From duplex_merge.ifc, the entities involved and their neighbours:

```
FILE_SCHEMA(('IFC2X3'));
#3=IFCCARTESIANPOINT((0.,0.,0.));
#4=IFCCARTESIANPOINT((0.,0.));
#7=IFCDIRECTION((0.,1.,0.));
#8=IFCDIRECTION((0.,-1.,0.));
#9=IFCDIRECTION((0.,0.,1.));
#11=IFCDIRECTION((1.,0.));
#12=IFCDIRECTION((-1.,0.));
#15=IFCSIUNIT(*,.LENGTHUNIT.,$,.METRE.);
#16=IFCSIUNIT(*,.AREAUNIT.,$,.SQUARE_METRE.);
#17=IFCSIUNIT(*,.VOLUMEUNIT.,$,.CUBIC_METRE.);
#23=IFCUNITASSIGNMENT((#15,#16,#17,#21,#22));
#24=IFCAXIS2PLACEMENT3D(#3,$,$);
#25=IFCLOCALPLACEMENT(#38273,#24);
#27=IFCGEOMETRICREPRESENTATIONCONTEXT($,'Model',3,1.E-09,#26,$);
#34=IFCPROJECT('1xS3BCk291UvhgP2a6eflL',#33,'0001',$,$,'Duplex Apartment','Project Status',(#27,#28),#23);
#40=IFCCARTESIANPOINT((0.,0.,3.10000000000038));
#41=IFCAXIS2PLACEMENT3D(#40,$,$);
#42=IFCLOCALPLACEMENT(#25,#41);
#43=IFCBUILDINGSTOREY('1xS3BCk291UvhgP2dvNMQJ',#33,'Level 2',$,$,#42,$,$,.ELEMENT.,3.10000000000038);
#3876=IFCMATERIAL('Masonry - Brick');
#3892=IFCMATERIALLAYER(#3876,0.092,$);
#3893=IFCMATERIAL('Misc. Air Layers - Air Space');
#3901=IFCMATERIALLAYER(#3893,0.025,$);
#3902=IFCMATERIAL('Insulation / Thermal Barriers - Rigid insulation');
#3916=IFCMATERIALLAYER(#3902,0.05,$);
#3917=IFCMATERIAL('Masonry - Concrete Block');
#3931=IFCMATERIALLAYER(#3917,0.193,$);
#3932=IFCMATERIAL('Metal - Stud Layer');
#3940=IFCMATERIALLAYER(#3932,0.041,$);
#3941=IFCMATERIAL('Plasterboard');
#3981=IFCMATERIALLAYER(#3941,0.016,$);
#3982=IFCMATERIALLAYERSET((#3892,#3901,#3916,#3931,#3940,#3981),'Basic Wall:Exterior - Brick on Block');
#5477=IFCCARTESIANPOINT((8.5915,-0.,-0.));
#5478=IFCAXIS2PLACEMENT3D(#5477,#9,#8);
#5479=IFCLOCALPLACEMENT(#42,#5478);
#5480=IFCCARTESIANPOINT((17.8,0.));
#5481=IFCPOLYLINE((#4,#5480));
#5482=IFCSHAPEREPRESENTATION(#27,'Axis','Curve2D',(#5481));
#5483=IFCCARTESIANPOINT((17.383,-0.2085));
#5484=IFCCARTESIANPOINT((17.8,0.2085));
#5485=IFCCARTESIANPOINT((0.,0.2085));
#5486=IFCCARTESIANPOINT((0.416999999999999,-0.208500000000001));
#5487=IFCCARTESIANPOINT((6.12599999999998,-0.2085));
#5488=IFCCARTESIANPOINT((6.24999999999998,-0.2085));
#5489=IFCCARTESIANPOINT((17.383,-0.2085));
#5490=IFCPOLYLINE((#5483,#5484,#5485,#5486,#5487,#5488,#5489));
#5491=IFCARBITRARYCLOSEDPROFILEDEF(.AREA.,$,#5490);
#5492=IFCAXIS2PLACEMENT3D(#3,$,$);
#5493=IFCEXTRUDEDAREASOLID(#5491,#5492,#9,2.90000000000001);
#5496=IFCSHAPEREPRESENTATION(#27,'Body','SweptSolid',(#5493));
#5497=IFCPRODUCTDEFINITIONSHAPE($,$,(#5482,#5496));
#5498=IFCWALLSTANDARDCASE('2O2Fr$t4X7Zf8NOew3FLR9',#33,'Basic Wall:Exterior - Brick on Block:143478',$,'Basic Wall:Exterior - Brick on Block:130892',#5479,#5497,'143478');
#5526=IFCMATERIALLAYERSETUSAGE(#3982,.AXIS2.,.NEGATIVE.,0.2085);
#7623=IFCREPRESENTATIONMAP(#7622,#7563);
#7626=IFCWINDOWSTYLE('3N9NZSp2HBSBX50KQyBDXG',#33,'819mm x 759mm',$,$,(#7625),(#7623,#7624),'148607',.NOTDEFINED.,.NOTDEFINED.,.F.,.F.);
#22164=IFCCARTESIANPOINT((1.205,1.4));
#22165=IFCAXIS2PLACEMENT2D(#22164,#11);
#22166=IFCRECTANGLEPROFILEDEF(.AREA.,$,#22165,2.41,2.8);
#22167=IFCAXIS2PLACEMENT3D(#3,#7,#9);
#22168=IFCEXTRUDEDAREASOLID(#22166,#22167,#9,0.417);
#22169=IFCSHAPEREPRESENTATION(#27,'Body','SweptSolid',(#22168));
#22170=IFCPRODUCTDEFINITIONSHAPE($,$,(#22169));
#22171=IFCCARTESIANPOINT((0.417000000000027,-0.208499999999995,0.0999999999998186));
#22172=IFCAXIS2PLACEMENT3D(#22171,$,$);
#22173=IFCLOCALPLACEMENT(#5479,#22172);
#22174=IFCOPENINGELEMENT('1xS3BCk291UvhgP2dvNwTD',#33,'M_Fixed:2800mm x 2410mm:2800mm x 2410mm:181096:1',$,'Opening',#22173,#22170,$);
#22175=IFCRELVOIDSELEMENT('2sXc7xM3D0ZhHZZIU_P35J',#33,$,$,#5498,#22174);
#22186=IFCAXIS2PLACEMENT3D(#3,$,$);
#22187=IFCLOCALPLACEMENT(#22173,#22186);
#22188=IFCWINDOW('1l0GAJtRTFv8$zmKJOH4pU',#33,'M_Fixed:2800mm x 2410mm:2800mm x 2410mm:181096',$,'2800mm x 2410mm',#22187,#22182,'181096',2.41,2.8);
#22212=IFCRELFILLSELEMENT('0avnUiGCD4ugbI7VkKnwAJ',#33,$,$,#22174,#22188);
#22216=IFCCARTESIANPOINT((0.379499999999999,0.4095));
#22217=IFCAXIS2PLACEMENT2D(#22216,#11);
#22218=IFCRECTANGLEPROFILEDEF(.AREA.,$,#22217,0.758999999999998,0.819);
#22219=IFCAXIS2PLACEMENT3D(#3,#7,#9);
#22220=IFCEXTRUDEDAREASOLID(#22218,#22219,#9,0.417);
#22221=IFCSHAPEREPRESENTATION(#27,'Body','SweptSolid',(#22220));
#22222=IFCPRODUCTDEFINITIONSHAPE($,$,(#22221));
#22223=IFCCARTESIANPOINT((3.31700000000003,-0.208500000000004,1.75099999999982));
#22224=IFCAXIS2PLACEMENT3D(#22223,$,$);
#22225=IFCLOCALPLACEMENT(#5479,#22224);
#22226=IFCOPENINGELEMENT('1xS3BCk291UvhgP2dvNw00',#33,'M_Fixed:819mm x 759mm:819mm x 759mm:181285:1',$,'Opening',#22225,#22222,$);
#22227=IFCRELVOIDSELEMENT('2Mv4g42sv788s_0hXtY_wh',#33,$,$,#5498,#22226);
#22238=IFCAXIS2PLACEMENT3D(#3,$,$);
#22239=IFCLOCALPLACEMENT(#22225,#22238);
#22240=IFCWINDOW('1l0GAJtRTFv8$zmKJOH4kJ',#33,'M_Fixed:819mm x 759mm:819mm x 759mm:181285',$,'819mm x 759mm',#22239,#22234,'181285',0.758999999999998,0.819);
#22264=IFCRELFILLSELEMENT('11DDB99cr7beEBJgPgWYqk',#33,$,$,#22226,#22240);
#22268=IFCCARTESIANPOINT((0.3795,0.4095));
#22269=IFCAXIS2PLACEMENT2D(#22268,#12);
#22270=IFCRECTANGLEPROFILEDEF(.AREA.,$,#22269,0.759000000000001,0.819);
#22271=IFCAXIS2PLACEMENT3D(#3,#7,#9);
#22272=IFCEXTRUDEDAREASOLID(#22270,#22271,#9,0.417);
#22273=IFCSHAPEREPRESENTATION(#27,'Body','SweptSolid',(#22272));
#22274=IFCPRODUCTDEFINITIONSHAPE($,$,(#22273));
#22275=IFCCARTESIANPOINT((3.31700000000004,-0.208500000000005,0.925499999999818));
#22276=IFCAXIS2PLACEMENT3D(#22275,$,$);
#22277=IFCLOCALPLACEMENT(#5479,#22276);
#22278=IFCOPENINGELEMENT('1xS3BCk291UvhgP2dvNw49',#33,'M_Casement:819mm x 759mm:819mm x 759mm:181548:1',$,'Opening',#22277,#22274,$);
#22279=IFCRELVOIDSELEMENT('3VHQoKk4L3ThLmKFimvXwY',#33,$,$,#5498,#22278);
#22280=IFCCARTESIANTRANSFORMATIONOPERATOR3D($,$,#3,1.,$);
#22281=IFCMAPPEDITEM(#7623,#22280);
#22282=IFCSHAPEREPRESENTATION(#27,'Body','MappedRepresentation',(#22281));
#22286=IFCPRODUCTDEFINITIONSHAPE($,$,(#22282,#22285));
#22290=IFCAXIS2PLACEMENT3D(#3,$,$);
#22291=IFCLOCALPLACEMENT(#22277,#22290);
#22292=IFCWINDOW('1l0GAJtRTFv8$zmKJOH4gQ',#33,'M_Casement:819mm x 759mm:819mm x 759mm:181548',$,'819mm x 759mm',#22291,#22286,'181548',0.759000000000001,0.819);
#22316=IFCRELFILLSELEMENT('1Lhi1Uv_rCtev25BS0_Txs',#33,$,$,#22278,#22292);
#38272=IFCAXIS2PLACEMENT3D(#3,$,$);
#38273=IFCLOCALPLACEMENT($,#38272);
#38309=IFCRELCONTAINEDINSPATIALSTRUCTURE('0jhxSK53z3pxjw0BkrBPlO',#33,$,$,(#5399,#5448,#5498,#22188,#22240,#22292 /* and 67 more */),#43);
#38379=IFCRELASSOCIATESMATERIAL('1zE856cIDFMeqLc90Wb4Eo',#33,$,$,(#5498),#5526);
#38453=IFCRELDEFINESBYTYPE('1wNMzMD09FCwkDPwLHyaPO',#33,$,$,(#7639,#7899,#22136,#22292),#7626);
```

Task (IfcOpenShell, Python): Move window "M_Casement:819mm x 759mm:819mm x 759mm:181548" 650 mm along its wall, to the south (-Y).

```python
import ifcopenshell
import ifcopenshell.api.geometry
import ifcopenshell.util.placement

model = ifcopenshell.open("duplex_merge.ifc")

window = model.by_guid("1l0GAJtRTFv8$zmKJOH4gQ")
opening = window.FillsVoids[0].RelatingOpeningElement
wall = opening.VoidsElements[0].RelatingBuildingElement

wall_matrix = ifcopenshell.util.placement.get_local_placement(wall.ObjectPlacement)
shift = wall_matrix[:3, 0] * 0.65
before = ifcopenshell.util.placement.get_local_placement(window.ObjectPlacement)[:3, 3].copy()

# The window is placed relative to its opening, so it follows when the opening moves.
matrix = ifcopenshell.util.placement.get_local_placement(opening.ObjectPlacement)
matrix[:3, 3] += shift
ifcopenshell.api.geometry.edit_object_placement(
    model, product=opening, matrix=matrix, is_si=False, should_transform_children=True
)

after = ifcopenshell.util.placement.get_local_placement(window.ObjectPlacement)[:3, 3]
print("window moved by", (after - before).round(3) + 0.0)

model.write("duplex_merge_v2.ifc")
```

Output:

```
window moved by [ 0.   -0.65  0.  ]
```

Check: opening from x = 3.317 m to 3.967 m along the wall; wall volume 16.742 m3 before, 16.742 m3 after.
